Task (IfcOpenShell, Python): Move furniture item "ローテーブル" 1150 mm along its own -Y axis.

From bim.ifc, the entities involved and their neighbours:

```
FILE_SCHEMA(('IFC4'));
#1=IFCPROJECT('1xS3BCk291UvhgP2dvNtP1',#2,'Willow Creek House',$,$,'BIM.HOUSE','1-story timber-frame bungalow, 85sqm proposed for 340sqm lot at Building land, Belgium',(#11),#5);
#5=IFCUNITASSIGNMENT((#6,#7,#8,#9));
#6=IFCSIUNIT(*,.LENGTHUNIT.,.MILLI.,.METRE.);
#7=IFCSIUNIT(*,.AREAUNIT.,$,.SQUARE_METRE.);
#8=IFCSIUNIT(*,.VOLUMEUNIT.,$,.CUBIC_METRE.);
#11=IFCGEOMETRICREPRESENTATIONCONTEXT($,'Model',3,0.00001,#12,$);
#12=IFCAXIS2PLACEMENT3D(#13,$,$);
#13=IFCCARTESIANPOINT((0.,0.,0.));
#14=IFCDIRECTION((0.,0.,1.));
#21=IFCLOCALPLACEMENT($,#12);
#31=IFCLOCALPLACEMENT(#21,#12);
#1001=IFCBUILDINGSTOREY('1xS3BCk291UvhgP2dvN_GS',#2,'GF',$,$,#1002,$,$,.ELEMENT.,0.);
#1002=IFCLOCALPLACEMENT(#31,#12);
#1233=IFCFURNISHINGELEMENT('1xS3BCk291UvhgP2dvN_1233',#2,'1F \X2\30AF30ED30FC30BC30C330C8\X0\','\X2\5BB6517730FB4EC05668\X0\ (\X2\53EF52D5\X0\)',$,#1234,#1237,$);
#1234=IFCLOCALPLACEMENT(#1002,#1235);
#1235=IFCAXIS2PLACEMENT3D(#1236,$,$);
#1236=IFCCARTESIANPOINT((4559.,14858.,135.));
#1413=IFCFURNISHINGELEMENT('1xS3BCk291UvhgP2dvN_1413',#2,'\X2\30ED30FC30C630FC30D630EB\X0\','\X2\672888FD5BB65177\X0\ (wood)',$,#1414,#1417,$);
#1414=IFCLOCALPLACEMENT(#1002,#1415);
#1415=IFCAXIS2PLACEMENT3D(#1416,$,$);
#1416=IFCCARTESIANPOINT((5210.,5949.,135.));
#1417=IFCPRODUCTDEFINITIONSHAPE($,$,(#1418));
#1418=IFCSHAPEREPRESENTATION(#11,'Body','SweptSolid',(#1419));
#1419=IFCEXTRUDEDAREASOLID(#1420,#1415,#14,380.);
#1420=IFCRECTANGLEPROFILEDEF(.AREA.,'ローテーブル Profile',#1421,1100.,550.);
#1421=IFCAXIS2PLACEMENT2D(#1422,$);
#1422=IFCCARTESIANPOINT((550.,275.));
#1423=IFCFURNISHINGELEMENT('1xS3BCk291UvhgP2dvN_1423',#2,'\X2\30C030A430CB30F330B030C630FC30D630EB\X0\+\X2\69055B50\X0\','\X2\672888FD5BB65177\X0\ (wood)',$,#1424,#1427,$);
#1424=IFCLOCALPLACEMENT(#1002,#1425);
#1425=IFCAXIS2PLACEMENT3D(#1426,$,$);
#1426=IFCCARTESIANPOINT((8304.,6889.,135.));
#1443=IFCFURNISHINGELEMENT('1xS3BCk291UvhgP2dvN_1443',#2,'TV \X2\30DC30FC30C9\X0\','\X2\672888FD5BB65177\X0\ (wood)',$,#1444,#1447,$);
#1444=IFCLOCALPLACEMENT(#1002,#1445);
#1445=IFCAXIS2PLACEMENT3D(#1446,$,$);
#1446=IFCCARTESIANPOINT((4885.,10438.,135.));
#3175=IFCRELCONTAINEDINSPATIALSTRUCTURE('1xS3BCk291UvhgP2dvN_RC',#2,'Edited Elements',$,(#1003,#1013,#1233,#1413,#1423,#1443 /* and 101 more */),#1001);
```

```python
import ifcopenshell
import ifcopenshell.api.geometry
import ifcopenshell.util.placement
import ifcopenshell.util.unit

model = ifcopenshell.open("bim.ifc")
unit_scale = ifcopenshell.util.unit.calculate_unit_scale(model)

item = model.by_guid("1xS3BCk291UvhgP2dvN_1413")
matrix = ifcopenshell.util.placement.get_local_placement(item.ObjectPlacement)
matrix[:3, 3] -= matrix[:3, 1] * 1.15 / unit_scale
ifcopenshell.api.geometry.edit_object_placement(model, product=item, matrix=matrix, is_si=False)

print(ifcopenshell.util.placement.get_local_placement(item.ObjectPlacement).round(3) + 0.0)

model.write("bim_updated.ifc")
```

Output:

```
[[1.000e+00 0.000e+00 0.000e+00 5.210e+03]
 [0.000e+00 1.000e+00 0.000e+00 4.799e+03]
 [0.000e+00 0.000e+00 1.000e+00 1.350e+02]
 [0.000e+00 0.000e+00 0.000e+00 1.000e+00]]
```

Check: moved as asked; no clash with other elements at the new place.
